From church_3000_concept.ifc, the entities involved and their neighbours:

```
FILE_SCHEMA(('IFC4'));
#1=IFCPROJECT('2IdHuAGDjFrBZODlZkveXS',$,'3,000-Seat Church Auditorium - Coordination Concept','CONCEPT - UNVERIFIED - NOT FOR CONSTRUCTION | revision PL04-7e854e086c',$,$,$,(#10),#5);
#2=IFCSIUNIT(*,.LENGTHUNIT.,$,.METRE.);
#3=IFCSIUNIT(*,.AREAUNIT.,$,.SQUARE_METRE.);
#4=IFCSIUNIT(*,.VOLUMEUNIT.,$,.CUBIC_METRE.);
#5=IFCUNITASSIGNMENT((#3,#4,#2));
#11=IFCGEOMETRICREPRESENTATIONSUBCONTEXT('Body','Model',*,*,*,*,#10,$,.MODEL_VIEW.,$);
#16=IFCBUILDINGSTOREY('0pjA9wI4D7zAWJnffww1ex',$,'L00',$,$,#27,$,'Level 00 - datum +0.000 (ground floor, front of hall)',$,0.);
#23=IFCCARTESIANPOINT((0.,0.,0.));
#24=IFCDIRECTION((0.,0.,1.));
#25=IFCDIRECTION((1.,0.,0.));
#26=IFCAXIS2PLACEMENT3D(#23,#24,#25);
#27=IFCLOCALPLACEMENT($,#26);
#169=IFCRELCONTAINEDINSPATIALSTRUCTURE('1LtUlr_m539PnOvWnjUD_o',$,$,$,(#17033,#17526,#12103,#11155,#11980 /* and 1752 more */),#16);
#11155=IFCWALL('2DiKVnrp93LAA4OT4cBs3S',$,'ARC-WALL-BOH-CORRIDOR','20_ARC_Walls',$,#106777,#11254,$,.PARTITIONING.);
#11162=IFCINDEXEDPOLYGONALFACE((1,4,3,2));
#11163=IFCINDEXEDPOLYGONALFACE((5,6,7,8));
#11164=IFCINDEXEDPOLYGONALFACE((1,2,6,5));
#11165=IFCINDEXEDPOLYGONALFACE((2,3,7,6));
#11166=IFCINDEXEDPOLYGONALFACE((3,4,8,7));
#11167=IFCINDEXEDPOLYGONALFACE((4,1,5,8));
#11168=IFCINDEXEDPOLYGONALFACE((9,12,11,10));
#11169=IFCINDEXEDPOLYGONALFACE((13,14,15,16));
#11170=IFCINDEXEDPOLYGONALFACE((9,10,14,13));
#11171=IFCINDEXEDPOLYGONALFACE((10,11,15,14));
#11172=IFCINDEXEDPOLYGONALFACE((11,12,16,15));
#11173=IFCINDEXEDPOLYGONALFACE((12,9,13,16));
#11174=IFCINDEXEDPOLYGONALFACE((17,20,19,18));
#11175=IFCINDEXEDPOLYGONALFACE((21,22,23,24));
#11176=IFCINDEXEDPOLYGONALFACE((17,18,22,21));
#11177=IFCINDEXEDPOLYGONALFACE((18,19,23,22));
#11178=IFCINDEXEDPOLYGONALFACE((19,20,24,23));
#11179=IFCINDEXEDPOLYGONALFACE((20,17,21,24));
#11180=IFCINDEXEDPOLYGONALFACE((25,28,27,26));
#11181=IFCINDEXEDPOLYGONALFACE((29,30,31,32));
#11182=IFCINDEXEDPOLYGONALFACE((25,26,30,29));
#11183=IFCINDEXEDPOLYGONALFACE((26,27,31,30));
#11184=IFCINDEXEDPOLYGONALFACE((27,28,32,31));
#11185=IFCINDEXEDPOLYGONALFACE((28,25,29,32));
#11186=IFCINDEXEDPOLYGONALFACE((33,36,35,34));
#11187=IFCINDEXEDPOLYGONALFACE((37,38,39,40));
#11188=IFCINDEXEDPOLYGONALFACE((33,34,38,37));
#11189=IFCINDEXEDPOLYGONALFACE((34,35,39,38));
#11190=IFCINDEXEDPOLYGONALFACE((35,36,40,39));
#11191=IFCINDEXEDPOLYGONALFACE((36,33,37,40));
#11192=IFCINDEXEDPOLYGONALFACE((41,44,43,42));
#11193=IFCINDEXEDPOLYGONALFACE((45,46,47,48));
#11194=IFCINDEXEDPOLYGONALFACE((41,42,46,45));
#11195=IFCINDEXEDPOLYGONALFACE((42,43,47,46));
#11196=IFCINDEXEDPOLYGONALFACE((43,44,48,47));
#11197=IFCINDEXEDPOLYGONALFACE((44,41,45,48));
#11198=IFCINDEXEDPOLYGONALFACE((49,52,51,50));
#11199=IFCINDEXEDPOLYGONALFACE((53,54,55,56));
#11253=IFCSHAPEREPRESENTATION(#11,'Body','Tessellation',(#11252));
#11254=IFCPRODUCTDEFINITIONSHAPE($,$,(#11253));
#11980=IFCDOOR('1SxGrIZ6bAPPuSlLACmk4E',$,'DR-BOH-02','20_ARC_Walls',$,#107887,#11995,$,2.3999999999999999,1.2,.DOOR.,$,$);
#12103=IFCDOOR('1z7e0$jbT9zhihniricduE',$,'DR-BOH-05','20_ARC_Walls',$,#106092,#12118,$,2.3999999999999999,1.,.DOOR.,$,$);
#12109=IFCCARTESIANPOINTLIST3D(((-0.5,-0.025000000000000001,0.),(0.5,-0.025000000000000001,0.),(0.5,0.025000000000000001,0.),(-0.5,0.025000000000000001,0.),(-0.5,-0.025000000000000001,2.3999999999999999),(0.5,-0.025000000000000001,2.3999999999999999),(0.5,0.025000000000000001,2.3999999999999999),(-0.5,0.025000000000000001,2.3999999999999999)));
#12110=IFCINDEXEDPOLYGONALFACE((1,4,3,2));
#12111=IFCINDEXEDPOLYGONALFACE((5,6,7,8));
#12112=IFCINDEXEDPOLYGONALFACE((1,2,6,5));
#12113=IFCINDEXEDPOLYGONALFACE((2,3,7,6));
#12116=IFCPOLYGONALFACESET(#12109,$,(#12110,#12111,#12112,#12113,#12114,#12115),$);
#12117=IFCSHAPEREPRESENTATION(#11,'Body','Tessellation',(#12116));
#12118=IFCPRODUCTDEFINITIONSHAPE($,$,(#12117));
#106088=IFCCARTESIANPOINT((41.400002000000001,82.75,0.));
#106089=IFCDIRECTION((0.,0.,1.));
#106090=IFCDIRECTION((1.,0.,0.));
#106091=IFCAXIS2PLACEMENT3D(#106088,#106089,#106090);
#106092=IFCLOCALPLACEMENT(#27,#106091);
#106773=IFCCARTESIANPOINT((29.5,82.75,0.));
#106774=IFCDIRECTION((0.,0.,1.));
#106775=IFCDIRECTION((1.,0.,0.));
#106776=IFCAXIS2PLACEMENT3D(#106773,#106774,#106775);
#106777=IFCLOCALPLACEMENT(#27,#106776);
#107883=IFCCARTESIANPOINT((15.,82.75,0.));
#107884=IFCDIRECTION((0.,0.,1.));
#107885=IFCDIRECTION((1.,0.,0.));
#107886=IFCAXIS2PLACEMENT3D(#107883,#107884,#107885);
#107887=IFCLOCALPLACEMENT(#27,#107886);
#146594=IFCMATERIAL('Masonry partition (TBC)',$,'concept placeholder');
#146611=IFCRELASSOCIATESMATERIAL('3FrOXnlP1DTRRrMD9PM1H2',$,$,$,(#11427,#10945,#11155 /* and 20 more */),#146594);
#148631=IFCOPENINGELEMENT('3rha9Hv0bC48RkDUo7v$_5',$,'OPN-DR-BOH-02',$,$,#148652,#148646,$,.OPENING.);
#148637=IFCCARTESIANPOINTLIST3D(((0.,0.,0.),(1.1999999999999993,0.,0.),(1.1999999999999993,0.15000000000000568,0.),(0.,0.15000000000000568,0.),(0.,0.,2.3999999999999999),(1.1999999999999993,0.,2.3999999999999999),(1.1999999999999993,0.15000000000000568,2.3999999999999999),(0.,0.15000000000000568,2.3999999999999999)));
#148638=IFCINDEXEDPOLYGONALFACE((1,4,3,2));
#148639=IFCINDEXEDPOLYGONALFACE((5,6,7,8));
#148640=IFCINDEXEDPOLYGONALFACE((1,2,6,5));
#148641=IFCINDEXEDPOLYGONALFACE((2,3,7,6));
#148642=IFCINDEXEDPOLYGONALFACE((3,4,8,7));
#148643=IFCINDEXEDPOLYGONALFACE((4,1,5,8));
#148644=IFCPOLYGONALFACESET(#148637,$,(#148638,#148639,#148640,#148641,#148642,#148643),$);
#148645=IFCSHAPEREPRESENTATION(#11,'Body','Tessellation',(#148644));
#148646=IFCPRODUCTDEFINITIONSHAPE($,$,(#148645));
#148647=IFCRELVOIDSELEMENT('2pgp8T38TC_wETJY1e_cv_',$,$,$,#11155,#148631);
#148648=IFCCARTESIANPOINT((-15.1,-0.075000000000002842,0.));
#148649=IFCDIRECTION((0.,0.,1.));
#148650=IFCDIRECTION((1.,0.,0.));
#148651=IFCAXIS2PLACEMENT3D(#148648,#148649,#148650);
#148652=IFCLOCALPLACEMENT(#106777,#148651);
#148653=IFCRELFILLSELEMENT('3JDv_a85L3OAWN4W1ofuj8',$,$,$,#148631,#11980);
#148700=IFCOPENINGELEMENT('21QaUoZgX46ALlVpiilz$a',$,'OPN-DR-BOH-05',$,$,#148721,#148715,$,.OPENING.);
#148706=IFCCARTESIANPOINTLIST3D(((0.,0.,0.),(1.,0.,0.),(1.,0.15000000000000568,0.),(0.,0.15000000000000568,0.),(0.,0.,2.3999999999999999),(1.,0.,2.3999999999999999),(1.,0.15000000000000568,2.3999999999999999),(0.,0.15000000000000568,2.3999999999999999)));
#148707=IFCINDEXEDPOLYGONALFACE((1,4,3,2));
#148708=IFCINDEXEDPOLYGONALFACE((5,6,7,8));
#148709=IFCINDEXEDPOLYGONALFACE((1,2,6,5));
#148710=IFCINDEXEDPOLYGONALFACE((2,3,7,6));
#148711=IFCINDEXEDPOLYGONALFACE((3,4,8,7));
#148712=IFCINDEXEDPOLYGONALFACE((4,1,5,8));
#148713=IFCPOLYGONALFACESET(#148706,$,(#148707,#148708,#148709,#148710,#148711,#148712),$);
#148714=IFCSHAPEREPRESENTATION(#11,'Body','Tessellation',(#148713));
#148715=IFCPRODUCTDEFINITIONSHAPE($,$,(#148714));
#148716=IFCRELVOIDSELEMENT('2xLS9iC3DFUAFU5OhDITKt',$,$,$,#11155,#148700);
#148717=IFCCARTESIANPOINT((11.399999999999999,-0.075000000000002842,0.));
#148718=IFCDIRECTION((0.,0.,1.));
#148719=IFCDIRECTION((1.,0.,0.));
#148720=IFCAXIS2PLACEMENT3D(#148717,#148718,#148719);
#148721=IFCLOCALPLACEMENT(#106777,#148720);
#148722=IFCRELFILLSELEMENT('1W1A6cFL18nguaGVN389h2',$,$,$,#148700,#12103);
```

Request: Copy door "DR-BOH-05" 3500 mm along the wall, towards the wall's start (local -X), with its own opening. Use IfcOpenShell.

```python
import ifcopenshell
import ifcopenshell.api.feature
import ifcopenshell.api.geometry
import ifcopenshell.api.root
import ifcopenshell.geom
import ifcopenshell.util.element
import ifcopenshell.util.placement
import ifcopenshell.util.shape
import ifcopenshell.util.unit

model = ifcopenshell.open("church_3000_concept.ifc")
unit_scale = ifcopenshell.util.unit.calculate_unit_scale(model)
settings = ifcopenshell.geom.settings()


def volume(element):
    """Net volume in cubic metres, openings subtracted."""
    shape = ifcopenshell.geom.create_shape(settings, element)
    return ifcopenshell.util.shape.get_volume(shape.geometry)


door = model.by_id(12103)
opening = door.FillsVoids[0].RelatingOpeningElement
wall = opening.VoidsElements[0].RelatingBuildingElement
before = volume(wall)
shift = ifcopenshell.util.placement.get_local_placement(wall.ObjectPlacement)[:3, 0] * -3.5 / unit_scale

# copy_class copies the void relationship, type, container and properties, but no geometry.
new_opening = ifcopenshell.api.root.copy_class(model, product=opening)
new_opening.Representation = ifcopenshell.util.element.copy_deep(
    model, opening.Representation, exclude=["IfcGeometricRepresentationContext", "IfcRepresentationMap"]
)
new_door = ifcopenshell.api.root.copy_class(model, product=door)
new_door.Representation = ifcopenshell.util.element.copy_deep(
    model, door.Representation, exclude=["IfcGeometricRepresentationContext", "IfcRepresentationMap"]
)
ifcopenshell.api.feature.add_filling(model, opening=new_opening, element=new_door)

for old, new in ((opening, new_opening), (door, new_door)):
    matrix = ifcopenshell.util.placement.get_local_placement(old.ObjectPlacement)
    matrix[:3, 3] += shift
    ifcopenshell.api.geometry.edit_object_placement(model, product=new, matrix=matrix, is_si=False)

after = volume(wall)

print(f"wall volume {before:.3f} -> {after:.3f} m3")

model.write("church_3000_concept-out.ifc")
```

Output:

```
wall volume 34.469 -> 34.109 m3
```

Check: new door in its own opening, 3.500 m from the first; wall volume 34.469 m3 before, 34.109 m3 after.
